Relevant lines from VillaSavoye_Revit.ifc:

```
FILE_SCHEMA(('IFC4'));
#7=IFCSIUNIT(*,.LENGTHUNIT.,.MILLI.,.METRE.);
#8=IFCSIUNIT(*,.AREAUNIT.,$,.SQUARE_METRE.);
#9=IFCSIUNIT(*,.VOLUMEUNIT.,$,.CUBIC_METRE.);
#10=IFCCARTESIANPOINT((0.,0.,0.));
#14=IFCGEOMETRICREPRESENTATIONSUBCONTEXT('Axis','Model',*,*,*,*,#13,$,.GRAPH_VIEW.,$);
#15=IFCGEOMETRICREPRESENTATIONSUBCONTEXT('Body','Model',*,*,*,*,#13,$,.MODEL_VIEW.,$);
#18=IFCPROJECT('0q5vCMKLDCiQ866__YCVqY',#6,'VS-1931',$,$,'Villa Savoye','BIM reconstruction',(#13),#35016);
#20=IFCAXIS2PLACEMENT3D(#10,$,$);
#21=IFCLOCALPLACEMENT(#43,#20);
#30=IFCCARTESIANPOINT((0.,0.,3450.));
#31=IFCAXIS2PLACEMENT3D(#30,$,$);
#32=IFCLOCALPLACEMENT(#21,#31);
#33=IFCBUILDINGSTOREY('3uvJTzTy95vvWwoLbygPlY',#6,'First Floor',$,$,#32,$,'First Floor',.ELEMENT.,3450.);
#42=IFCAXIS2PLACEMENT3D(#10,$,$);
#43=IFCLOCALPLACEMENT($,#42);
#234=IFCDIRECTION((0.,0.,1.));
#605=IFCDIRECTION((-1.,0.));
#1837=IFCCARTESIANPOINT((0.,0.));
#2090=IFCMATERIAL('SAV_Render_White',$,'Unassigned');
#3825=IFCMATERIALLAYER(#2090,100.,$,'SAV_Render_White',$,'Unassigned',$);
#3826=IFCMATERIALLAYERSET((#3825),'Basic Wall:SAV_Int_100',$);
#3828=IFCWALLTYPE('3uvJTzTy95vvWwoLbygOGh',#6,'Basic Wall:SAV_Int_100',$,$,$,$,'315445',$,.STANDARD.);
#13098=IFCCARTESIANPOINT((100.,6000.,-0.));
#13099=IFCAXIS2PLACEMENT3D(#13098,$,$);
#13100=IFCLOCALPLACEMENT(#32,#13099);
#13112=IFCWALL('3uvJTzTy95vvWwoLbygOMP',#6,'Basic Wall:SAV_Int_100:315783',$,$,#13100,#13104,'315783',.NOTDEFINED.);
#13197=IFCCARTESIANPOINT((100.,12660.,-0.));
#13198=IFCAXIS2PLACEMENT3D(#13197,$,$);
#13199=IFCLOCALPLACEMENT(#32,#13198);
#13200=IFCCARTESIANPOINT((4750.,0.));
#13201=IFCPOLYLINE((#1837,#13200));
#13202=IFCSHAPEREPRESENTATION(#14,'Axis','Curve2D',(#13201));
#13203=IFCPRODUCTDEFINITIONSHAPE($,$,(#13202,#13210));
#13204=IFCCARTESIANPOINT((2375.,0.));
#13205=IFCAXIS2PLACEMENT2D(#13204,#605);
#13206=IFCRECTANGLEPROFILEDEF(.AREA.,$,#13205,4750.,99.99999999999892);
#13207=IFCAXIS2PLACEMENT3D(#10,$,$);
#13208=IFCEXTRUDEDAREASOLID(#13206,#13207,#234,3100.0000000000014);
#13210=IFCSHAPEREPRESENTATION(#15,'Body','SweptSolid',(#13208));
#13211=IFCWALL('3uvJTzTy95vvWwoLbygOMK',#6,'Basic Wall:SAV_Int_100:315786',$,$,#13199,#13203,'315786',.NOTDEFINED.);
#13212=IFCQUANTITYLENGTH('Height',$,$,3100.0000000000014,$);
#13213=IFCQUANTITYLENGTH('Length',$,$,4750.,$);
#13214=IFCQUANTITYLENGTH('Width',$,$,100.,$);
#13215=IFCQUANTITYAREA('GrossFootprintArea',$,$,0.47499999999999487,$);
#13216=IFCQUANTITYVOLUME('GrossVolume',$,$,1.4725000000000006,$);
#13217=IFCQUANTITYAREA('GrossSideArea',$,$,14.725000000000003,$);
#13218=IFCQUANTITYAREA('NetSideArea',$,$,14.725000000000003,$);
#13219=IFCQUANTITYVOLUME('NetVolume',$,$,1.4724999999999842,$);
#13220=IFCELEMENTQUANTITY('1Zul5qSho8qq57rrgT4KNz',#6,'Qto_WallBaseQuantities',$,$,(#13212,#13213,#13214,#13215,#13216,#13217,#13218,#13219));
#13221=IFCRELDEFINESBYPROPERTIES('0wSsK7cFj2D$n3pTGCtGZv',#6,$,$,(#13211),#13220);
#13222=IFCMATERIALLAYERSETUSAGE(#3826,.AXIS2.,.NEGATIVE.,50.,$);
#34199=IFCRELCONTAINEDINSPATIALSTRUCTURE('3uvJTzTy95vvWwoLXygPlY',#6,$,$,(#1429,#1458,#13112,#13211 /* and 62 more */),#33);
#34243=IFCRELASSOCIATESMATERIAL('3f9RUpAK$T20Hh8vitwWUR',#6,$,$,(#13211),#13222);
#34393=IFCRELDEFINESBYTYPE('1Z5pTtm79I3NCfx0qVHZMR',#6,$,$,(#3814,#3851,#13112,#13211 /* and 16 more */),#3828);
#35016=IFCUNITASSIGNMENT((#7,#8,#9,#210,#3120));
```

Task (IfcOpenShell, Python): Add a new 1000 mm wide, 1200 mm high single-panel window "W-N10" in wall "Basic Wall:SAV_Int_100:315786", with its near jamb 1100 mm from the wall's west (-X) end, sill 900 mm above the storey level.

```python
import numpy as np
import ifcopenshell
import ifcopenshell.api.feature
import ifcopenshell.api.geometry
import ifcopenshell.api.pset
import ifcopenshell.api.root
import ifcopenshell.api.spatial
import ifcopenshell.geom
import ifcopenshell.util.element
import ifcopenshell.util.placement
import ifcopenshell.util.representation
import ifcopenshell.util.shape
import ifcopenshell.util.unit

model = ifcopenshell.open("VillaSavoye_Revit.ifc")
unit_scale = ifcopenshell.util.unit.calculate_unit_scale(model)
area_scale = ifcopenshell.util.unit.calculate_unit_scale(model, "AREAUNIT")
volume_scale = ifcopenshell.util.unit.calculate_unit_scale(model, "VOLUMEUNIT")
settings = ifcopenshell.geom.settings()


def volume(element):
    """Net volume in cubic metres, openings subtracted."""
    shape = ifcopenshell.geom.create_shape(settings, element)
    return ifcopenshell.util.shape.get_volume(shape.geometry)


wall = model.by_id(13211)
storey = ifcopenshell.util.element.get_container(wall, ifc_class="IfcBuildingStorey")
context = ifcopenshell.util.representation.get_context(model, "Model", "Body", "MODEL_VIEW")
before = volume(wall)

width, height, from_end, sill = 1, 1.2, 1.1, 0.9  # metres

# The wall runs along its own X axis, and the end named is its -X end.
wall_shape = ifcopenshell.geom.create_shape(settings, wall)
x, y, z = ifcopenshell.util.shape.get_vertices(wall_shape.geometry).T
start = x.min() + from_end
face, thickness = float(y.min()), float(y.max() - y.min())
wall_matrix = ifcopenshell.util.placement.get_local_placement(wall.ObjectPlacement)
level = ifcopenshell.util.placement.get_local_placement(storey.ObjectPlacement)[2, 3]


def in_wall(x, y):
    """Placement at x, y metres in the wall's axes, at sill height."""
    matrix = wall_matrix.copy()
    matrix[:, 3] = wall_matrix @ np.array([x / unit_scale, y / unit_scale, 0.0, 1.0])
    matrix[2, 3] = level + sill / unit_scale
    return matrix


# Opening: a box that overshoots both wall faces by 50 mm.
opening = ifcopenshell.api.root.create_entity(model, ifc_class="IfcOpeningElement", predefined_type="OPENING")
box = ifcopenshell.api.geometry.add_wall_representation(
    model, context=context, length=width, height=height, thickness=thickness + 0.1
)
ifcopenshell.api.geometry.assign_representation(model, product=opening, representation=box)
ifcopenshell.api.geometry.edit_object_placement(model, product=opening, matrix=in_wall(start, face - 0.05), is_si=False)
ifcopenshell.api.feature.add_feature(model, feature=opening, element=wall)

window = ifcopenshell.api.root.create_entity(model, ifc_class="IfcWindow", name="W-N10", predefined_type="WINDOW")
window.OverallWidth, window.OverallHeight = width / unit_scale, height / unit_scale
window.PartitioningType = "SINGLE_PANEL"
body = ifcopenshell.api.geometry.add_window_representation(
    model,
    context=context,
    overall_width=window.OverallWidth,
    overall_height=window.OverallHeight,
    partition_type="SINGLE_PANEL",
)
ifcopenshell.api.geometry.assign_representation(model, product=window, representation=body)
ifcopenshell.api.spatial.assign_container(model, products=[window], relating_structure=storey)
ifcopenshell.api.feature.add_filling(model, opening=opening, element=window)

# Centre the window in the wall's thickness.
ifcopenshell.api.geometry.edit_object_placement(model, product=window, matrix=in_wall(start, face), is_si=False)
window_shape = ifcopenshell.geom.create_shape(settings, window)
depth = ifcopenshell.util.shape.get_vertices(window_shape.geometry)[:, 1]
offset = face + thickness / 2 - (depth.min() + depth.max()) / 2
ifcopenshell.api.geometry.edit_object_placement(model, product=window, matrix=in_wall(start, offset), is_si=False)

after = volume(wall)

# Update the wall's stored quantities.
qto = model.by_id(ifcopenshell.util.element.get_pset(wall, "Qto_WallBaseQuantities", should_inherit=False)["id"])
ifcopenshell.api.pset.edit_qto(model, qto=qto, properties={
    "NetSideArea": after / thickness / area_scale,
    "NetVolume": after / volume_scale,
})

print(f"wall volume {before:.3f} -> {after:.3f} m3")

model.write("VillaSavoye_Revit-out.ifc")
```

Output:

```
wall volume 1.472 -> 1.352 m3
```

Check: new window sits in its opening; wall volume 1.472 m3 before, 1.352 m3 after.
